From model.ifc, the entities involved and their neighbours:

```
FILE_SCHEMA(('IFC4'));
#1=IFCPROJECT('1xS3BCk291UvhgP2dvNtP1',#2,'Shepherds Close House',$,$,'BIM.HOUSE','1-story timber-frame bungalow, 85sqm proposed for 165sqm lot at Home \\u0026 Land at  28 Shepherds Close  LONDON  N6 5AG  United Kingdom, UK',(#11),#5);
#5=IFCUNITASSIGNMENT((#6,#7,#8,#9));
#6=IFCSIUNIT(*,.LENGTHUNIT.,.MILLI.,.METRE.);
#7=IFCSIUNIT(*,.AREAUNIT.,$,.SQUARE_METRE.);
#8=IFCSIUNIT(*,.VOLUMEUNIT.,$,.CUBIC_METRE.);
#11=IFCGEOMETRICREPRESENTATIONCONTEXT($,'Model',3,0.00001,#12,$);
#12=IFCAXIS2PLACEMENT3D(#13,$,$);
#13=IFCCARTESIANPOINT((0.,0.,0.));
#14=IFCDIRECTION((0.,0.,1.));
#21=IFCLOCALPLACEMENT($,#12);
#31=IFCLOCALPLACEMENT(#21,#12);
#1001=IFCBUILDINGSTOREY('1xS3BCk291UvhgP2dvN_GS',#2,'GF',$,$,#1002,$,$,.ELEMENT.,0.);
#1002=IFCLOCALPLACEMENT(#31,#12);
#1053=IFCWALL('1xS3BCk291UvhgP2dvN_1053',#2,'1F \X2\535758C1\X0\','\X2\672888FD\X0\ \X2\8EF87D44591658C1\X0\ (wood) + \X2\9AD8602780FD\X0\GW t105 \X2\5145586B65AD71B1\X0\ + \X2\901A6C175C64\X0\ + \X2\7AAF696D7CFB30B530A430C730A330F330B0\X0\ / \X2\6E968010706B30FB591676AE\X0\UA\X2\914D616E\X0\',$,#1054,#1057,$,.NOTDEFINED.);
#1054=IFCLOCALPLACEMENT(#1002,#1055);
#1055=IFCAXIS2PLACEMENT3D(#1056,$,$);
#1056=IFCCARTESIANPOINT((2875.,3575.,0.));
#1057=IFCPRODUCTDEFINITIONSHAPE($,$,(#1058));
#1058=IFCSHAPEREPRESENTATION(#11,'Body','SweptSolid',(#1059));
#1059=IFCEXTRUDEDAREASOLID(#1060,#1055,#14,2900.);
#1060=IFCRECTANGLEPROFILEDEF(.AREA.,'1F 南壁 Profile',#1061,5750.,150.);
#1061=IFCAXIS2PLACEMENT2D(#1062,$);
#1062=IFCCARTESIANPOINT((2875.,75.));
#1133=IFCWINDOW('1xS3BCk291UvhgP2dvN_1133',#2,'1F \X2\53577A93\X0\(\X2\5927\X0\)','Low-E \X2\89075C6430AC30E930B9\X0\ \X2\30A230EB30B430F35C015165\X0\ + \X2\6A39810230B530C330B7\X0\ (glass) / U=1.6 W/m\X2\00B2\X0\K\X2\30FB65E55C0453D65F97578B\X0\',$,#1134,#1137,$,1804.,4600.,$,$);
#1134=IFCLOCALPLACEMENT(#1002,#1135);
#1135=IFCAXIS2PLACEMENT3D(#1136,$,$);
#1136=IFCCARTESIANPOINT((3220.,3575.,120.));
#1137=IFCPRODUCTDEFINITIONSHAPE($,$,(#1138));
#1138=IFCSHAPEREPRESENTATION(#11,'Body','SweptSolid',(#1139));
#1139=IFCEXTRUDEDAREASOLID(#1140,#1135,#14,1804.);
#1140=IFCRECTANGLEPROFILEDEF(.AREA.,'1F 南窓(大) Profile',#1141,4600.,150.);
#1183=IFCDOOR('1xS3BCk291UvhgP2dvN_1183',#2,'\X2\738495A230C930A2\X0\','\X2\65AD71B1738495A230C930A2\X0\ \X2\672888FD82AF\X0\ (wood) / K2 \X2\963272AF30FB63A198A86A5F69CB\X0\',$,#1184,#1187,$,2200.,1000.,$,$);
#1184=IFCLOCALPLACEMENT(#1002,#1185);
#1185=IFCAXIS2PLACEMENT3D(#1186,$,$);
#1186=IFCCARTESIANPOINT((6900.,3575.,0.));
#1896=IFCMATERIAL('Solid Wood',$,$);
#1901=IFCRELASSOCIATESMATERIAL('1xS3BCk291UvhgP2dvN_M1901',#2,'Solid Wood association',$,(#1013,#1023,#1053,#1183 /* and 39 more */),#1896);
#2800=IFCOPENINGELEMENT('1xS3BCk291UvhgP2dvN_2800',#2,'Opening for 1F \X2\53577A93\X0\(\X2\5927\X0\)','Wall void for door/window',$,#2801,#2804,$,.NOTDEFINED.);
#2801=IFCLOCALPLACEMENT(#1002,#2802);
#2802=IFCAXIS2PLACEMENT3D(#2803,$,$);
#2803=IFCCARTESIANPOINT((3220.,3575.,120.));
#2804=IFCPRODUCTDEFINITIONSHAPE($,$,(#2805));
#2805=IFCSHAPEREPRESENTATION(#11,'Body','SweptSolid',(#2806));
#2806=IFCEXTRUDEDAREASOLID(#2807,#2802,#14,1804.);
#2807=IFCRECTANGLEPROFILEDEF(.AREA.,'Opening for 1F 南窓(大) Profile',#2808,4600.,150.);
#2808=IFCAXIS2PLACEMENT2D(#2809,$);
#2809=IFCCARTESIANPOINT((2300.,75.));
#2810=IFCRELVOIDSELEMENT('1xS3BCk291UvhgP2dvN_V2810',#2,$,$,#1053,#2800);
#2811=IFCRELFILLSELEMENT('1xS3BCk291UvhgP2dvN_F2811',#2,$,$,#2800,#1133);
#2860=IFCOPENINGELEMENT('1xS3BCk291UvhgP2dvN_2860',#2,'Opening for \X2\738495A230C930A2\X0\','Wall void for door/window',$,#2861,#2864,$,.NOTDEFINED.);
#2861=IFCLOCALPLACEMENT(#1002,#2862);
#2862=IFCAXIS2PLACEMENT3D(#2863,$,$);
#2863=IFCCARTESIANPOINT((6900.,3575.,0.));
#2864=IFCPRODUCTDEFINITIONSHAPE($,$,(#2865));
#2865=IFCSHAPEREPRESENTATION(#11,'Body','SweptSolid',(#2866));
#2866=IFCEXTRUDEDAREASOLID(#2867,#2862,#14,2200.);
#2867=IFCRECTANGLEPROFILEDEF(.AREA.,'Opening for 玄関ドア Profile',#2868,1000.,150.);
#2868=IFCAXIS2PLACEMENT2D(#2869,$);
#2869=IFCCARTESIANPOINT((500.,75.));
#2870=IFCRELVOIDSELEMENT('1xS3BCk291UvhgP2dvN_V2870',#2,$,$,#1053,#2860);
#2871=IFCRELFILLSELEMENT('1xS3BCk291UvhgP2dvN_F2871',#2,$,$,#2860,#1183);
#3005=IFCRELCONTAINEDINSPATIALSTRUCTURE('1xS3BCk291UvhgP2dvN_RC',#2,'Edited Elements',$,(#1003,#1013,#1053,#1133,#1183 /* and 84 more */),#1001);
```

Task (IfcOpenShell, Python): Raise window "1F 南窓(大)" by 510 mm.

```python
import numpy as np
import ifcopenshell
import ifcopenshell.api.geometry
import ifcopenshell.util.placement
import ifcopenshell.util.unit

model = ifcopenshell.open("model.ifc")
unit_scale = ifcopenshell.util.unit.calculate_unit_scale(model)

window = model.by_guid("1xS3BCk291UvhgP2dvN_1133")
opening = window.FillsVoids[0].RelatingOpeningElement
dz = 510.0

shift = np.array([0.0, 0.0, dz])
# The window is not placed relative to its opening, so move both.
for product in (opening, window):
    matrix = ifcopenshell.util.placement.get_local_placement(product.ObjectPlacement)
    matrix[:3, 3] += shift
    ifcopenshell.api.geometry.edit_object_placement(model, product=product, matrix=matrix, is_si=False)

print(f"moved by {dz * unit_scale:+.3f} m")

model.write("model_v2.ifc")
```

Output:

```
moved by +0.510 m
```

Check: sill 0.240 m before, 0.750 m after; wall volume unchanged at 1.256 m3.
